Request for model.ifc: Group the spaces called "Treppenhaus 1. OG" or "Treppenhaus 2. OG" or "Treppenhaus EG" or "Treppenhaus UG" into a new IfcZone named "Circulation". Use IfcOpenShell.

First a look at what the model holds.

```python
import ifcopenshell

model = ifcopenshell.open("model.ifc")
print(model.schema)
seen = {}
for space in model.by_type("IfcSpace"):
    seen[space.Name] = seen.get(space.Name, 0) + 1
for name, count in sorted(seen.items(), key=str):
    print(count, "x", name)
print("zones:", [z.Name for z in model.by_type("IfcZone")][:20])
```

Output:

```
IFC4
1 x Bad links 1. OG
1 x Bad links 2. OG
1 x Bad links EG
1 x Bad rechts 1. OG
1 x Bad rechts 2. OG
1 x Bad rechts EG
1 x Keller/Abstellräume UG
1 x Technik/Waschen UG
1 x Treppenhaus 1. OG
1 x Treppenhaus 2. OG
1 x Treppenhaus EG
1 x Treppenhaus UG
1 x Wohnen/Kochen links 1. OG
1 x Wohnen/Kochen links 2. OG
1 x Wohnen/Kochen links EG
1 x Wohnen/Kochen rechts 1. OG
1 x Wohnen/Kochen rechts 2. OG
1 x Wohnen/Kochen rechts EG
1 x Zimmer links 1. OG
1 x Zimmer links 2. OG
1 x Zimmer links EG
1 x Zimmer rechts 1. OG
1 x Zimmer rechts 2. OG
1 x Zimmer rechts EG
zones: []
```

```python
import ifcopenshell
import ifcopenshell.api.group
import ifcopenshell.api.root

model = ifcopenshell.open("model.ifc")

names = {"Treppenhaus 1. OG", "Treppenhaus 2. OG", "Treppenhaus EG", "Treppenhaus UG"}
spaces = [s for s in model.by_type("IfcSpace") if s.Name in names]

zone = ifcopenshell.api.root.create_entity(model, ifc_class="IfcZone", name="Circulation")
ifcopenshell.api.group.assign_group(model, products=spaces, group=zone)
print(len(spaces), "spaces in", zone.Name)

model.write("model_updated.ifc")
```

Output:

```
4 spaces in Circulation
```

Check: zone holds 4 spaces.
